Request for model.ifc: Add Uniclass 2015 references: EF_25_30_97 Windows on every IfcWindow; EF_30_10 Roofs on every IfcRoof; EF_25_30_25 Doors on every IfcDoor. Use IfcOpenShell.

First a look at what the model holds.

```python
import ifcopenshell

model = ifcopenshell.open("model.ifc")
print(model.schema)
print("classifications:", [c.Name for c in model.by_type("IfcClassification")])
for ifc_class in ("IfcDoor", "IfcRoof", "IfcStair", "IfcWall", "IfcWindow"):
    print(ifc_class, len(model.by_type(ifc_class)))
```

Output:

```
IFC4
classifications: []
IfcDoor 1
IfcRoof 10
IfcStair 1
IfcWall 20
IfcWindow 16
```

```python
import ifcopenshell
import ifcopenshell.api.classification

model = ifcopenshell.open("model.ifc")

system = ifcopenshell.api.classification.add_classification(model, classification="Uniclass 2015")

codes = {
    "IfcWindow": ("EF_25_30_97", "Windows"),
    "IfcRoof": ("EF_30_10", "Roofs"),
    "IfcDoor": ("EF_25_30_25", "Doors"),
}
for ifc_class, (code, name) in codes.items():
    products = model.by_type(ifc_class)
    ifcopenshell.api.classification.add_reference(
        model, products=products, classification=system, identification=code, name=name
    )
    print(code, len(products))

model.write("model-out.ifc")
```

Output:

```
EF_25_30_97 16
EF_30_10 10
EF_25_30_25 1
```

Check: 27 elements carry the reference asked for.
